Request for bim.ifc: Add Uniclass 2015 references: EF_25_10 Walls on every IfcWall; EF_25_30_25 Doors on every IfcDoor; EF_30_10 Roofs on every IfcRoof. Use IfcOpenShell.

First a look at what the model holds.

```python
import ifcopenshell

model = ifcopenshell.open("bim.ifc")
print(model.schema)
print("classifications:", [c.Name for c in model.by_type("IfcClassification")])
for ifc_class in ("IfcDoor", "IfcRoof", "IfcStair", "IfcWall", "IfcWindow"):
    print(ifc_class, len(model.by_type(ifc_class)))
```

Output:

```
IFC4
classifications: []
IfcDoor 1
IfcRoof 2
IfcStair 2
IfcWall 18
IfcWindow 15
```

```python
import ifcopenshell
import ifcopenshell.api.classification

model = ifcopenshell.open("bim.ifc")

system = ifcopenshell.api.classification.add_classification(model, classification="Uniclass 2015")

codes = {
    "IfcWall": ("EF_25_10", "Walls"),
    "IfcDoor": ("EF_25_30_25", "Doors"),
    "IfcRoof": ("EF_30_10", "Roofs"),
}
for ifc_class, (code, name) in codes.items():
    products = model.by_type(ifc_class)
    ifcopenshell.api.classification.add_reference(
        model, products=products, classification=system, identification=code, name=name
    )
    print(code, len(products))

model.write("bim_rev.ifc")
```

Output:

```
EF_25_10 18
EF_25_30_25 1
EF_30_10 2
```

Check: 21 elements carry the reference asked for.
